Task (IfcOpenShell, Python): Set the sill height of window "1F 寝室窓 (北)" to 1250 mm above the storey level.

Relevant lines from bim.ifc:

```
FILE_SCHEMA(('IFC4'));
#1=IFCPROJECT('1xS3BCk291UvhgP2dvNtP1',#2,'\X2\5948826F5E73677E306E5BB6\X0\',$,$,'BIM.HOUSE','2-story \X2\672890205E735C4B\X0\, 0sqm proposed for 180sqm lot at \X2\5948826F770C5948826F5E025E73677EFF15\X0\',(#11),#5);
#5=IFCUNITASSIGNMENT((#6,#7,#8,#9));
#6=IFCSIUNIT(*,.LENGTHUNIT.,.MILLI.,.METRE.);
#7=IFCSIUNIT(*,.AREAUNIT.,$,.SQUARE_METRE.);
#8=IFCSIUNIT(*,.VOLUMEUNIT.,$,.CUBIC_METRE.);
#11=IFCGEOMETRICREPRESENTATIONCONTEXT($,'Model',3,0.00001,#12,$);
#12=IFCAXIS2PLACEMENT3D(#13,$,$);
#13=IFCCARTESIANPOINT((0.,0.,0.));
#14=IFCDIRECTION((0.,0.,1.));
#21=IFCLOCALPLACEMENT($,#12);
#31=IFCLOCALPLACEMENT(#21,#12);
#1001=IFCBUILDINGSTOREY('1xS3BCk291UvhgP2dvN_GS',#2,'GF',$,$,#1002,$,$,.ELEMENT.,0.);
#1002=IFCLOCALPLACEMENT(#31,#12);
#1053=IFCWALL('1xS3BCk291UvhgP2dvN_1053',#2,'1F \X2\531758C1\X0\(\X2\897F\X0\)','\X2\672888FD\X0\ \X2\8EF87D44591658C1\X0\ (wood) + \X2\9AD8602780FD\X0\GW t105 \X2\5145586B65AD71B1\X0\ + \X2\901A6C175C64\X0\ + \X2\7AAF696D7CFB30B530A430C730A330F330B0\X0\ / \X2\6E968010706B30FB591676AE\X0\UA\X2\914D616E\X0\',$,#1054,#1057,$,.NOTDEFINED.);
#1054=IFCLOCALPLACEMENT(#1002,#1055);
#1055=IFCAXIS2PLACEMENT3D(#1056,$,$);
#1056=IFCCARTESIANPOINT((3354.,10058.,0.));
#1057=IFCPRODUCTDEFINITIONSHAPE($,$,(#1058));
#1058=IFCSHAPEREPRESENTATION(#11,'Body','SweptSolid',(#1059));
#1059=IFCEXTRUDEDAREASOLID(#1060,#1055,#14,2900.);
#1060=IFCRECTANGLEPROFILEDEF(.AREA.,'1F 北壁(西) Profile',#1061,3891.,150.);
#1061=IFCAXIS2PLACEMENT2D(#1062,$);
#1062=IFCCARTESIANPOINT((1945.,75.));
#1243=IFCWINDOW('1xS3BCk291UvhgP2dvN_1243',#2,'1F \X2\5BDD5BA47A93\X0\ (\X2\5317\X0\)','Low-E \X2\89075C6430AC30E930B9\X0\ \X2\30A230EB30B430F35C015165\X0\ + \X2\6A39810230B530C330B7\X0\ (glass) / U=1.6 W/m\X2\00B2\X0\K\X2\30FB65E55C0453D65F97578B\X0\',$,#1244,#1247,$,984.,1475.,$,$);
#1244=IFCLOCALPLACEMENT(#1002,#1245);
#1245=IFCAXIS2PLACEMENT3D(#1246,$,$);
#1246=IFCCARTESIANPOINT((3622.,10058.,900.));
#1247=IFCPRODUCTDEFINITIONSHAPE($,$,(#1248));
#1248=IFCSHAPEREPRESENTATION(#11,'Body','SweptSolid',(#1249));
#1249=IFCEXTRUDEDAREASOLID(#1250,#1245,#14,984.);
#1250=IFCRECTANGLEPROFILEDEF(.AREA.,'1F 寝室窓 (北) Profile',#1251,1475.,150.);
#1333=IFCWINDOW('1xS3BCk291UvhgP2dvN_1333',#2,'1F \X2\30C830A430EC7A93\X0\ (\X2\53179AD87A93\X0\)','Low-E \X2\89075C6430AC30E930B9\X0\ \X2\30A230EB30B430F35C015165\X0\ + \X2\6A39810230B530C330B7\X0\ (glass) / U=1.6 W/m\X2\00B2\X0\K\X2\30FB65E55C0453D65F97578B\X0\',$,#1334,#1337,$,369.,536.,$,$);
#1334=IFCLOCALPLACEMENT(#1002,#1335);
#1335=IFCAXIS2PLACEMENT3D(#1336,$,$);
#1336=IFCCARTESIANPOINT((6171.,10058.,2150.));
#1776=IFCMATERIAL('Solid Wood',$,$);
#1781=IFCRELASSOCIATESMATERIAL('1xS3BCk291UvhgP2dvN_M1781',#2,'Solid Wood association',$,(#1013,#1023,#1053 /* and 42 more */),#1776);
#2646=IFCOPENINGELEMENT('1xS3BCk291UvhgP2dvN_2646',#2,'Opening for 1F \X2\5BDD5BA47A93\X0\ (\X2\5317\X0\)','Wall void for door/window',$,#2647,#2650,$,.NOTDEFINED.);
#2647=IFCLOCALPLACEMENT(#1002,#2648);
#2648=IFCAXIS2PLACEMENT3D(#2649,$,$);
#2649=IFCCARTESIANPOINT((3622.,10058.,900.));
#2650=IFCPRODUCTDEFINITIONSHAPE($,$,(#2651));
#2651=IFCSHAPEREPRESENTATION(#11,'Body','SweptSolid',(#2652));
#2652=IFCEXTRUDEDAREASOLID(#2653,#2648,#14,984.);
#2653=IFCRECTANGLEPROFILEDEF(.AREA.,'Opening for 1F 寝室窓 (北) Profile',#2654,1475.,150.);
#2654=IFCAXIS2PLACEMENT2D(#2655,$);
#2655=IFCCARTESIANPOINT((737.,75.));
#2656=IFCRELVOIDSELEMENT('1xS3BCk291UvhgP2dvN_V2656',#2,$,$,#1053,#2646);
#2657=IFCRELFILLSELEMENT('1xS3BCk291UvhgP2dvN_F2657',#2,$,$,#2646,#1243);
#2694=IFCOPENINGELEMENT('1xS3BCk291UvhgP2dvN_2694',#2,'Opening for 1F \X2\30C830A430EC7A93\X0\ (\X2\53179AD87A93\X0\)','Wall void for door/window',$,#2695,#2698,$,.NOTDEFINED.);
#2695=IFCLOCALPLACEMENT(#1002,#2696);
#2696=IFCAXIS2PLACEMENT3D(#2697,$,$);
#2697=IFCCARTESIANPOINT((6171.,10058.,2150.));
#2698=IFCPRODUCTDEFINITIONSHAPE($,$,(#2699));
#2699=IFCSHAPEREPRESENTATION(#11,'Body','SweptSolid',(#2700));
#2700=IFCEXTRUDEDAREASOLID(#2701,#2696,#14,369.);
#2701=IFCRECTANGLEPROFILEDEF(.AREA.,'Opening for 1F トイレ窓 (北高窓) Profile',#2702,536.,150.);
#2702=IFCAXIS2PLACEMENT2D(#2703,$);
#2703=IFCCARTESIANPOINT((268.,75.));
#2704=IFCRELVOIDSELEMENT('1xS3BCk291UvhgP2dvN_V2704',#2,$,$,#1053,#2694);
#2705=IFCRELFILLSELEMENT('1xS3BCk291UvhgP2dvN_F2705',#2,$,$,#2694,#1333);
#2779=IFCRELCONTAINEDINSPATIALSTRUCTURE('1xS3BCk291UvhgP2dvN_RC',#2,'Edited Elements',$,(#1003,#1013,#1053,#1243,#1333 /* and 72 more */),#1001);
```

```python
import numpy as np
import ifcopenshell
import ifcopenshell.api.geometry
import ifcopenshell.geom
import ifcopenshell.util.element
import ifcopenshell.util.placement
import ifcopenshell.util.shape
import ifcopenshell.util.unit

model = ifcopenshell.open("bim.ifc")
unit_scale = ifcopenshell.util.unit.calculate_unit_scale(model)

window = model.by_guid("1xS3BCk291UvhgP2dvN_1243")
opening = window.FillsVoids[0].RelatingOpeningElement
storey = ifcopenshell.util.element.get_container(window, ifc_class="IfcBuildingStorey")
level = ifcopenshell.util.placement.get_local_placement(storey.ObjectPlacement)[2, 3]

# The opening's origin need not be at the sill, so measure its lowest point.
shape = ifcopenshell.geom.create_shape(ifcopenshell.geom.settings(), opening)
bottom = ifcopenshell.util.shape.get_shape_bottom_elevation(shape, shape.geometry) / unit_scale
dz = level + 1.25 / unit_scale - bottom

shift = np.array([0.0, 0.0, dz])
# The window is not placed relative to its opening, so move both.
for product in (opening, window):
    matrix = ifcopenshell.util.placement.get_local_placement(product.ObjectPlacement)
    matrix[:3, 3] += shift
    ifcopenshell.api.geometry.edit_object_placement(model, product=product, matrix=matrix, is_si=False)

print(f"moved by {dz * unit_scale:+.3f} m")

model.write("bim_updated.ifc")
```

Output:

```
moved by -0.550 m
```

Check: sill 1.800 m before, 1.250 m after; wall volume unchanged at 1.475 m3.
